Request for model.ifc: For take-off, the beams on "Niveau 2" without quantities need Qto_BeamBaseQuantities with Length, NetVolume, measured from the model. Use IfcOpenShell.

First a look at what the model holds.

```python
import ifcopenshell
import ifcopenshell.util.element
import ifcopenshell.util.unit

model = ifcopenshell.open("model.ifc")
print(model.schema)
for unit_type in ("LENGTHUNIT", "AREAUNIT", "VOLUMEUNIT"):
    print(unit_type, ifcopenshell.util.unit.calculate_unit_scale(model, unit_type))
storey = next(s for s in model.by_type("IfcBuildingStorey") if s.Name == "Niveau 2")
beams = [e for e in ifcopenshell.util.element.get_decomposition(storey) if e.is_a("IfcBeam")]
for e in sorted(beams, key=lambda e: e.id()):
    print(e.id(), e.is_a(), e.Name, list(ifcopenshell.util.element.get_psets(e, qtos_only=True)), sep=" | ")
```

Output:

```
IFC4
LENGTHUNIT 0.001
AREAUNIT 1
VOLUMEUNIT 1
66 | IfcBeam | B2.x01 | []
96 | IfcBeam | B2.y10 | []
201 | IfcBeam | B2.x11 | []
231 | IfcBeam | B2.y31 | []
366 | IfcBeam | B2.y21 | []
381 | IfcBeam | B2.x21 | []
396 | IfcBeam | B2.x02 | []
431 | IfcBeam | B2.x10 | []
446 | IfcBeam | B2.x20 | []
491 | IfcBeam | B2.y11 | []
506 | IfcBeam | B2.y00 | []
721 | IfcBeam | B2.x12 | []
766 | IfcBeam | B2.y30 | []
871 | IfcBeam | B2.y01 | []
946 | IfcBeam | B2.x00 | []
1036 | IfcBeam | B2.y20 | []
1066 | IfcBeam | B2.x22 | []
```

```python
import ifcopenshell
import ifcopenshell.api.pset
import ifcopenshell.geom
import ifcopenshell.util.element
import ifcopenshell.util.shape
import ifcopenshell.util.unit

model = ifcopenshell.open("model.ifc")
unit_scale = ifcopenshell.util.unit.calculate_unit_scale(model)
volume_scale = ifcopenshell.util.unit.calculate_unit_scale(model, "VOLUMEUNIT")
settings = ifcopenshell.geom.settings()

storey = next(s for s in model.by_type("IfcBuildingStorey") if s.Name == "Niveau 2")
beams = [e for e in ifcopenshell.util.element.get_decomposition(storey) if e.is_a("IfcBeam")]

for e in sorted(beams, key=lambda e: e.id()):
    if ifcopenshell.util.element.get_psets(e, qtos_only=True, should_inherit=False):
        continue
    # Geometry comes back in metres, in the element's own axes.
    shape = ifcopenshell.geom.create_shape(settings, e)
    values = {
        "Length": ifcopenshell.util.shape.get_max_xyz(shape.geometry) / unit_scale,
        "NetVolume": ifcopenshell.util.shape.get_volume(shape.geometry) / volume_scale,
    }
    qto = ifcopenshell.api.pset.add_qto(model, product=e, name="Qto_BeamBaseQuantities")
    ifcopenshell.api.pset.edit_qto(model, qto=qto, properties=values)
    print(e.id(), {k: round(v, 3) for k, v in values.items()})

model.write("model_v2.ifc")
```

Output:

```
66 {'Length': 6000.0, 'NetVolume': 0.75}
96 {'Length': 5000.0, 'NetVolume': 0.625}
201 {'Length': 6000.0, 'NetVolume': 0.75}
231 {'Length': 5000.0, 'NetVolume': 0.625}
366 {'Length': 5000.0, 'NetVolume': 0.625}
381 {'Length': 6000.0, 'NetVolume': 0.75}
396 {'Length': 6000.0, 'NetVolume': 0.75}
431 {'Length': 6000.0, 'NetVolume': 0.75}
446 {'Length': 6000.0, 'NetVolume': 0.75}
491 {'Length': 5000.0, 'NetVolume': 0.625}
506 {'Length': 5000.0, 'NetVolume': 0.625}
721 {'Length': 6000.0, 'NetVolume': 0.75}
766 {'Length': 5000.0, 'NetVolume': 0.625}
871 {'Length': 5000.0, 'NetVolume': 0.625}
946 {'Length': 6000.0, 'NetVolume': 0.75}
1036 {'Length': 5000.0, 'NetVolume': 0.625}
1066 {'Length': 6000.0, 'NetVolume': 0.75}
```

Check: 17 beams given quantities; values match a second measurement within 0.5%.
